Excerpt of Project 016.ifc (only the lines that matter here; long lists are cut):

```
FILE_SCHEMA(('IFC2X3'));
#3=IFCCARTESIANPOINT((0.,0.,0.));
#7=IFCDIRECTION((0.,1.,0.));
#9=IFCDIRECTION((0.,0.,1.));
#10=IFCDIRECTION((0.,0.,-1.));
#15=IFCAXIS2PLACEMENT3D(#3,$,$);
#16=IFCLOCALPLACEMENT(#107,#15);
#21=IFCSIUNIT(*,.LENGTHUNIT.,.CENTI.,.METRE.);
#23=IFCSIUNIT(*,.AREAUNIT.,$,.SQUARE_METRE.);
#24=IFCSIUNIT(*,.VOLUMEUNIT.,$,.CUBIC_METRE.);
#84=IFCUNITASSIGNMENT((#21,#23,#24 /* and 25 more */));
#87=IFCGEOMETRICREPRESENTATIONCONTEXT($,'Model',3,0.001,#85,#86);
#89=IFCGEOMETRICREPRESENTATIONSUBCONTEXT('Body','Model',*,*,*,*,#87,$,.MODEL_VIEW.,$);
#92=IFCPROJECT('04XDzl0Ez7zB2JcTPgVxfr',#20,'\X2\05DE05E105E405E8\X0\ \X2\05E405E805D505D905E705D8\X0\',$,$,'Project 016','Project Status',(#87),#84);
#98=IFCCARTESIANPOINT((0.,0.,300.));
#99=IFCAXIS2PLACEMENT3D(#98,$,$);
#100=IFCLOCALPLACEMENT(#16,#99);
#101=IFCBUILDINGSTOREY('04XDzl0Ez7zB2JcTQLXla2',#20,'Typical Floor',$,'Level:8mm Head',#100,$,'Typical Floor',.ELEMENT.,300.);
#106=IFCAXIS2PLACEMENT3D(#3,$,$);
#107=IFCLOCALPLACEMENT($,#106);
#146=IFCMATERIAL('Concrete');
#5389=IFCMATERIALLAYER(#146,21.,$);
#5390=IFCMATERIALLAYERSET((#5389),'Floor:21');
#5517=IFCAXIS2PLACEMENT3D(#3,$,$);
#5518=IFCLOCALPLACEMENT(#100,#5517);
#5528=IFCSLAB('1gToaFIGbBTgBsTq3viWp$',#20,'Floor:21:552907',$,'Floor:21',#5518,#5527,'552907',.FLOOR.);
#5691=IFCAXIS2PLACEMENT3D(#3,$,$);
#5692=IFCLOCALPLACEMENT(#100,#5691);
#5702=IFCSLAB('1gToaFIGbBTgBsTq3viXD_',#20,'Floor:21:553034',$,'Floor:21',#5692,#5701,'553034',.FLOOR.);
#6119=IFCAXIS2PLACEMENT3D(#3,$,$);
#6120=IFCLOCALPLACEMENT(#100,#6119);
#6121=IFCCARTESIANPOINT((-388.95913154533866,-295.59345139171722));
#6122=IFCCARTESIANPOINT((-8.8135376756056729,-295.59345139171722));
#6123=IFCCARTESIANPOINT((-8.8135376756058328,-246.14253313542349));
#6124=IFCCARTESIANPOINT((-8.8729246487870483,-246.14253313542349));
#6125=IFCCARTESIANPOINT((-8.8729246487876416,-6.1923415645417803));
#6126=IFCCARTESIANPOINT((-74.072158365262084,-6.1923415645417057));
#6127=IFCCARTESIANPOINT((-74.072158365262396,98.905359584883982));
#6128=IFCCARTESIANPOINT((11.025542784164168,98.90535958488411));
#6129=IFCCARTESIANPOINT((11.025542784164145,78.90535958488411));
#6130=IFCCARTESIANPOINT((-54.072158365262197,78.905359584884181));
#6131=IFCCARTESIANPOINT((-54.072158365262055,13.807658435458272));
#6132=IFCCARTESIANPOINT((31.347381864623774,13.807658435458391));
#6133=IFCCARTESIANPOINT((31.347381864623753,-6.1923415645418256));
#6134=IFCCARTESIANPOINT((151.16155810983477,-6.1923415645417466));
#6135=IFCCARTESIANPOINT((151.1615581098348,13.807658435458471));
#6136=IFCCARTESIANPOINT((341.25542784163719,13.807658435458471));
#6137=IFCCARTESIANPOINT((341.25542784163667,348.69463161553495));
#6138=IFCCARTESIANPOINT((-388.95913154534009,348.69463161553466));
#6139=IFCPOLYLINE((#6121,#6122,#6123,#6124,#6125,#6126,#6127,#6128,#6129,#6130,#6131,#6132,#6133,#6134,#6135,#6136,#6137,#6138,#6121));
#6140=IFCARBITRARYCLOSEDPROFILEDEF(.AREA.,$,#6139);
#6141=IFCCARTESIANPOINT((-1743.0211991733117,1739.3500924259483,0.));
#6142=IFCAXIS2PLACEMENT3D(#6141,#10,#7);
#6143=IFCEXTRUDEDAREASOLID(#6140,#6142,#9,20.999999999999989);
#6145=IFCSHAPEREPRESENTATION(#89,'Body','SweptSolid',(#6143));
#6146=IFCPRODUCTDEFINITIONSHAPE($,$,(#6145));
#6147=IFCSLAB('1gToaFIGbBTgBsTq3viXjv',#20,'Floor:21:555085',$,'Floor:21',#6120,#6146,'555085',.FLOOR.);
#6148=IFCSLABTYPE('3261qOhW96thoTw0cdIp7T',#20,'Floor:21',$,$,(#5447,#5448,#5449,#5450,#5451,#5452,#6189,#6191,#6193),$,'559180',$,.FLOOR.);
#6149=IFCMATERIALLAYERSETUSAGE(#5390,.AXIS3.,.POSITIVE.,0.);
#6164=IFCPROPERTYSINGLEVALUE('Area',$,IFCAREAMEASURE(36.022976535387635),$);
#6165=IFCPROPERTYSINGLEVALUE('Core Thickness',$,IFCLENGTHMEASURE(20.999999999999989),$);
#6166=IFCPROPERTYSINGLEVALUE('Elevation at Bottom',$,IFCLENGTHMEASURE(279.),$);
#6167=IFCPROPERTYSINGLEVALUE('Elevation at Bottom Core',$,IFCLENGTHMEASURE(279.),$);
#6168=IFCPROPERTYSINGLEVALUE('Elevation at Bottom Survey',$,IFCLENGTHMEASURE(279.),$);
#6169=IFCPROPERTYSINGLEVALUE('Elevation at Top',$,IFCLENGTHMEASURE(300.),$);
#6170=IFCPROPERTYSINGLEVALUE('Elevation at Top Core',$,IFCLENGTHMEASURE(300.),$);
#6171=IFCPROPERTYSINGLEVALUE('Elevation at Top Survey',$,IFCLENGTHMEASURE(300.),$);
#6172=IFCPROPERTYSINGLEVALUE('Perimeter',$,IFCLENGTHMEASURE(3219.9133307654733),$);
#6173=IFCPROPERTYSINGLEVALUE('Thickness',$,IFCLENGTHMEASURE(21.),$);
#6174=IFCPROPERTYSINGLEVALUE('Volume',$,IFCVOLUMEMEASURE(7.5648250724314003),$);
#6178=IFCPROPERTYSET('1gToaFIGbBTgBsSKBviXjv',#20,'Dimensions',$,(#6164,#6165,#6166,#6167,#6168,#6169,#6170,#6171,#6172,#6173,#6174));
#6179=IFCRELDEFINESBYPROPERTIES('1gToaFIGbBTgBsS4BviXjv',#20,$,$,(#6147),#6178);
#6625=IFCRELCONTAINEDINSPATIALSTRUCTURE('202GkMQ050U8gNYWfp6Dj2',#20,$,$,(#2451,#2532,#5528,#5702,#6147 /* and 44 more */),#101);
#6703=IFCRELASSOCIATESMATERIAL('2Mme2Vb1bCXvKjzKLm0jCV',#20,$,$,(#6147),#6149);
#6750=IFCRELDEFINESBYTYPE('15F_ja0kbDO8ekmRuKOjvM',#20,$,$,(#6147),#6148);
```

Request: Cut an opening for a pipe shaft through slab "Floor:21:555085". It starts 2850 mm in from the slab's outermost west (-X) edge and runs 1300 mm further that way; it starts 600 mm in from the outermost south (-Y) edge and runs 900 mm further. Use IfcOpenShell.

```python
import numpy as np
import ifcopenshell
import ifcopenshell.api.feature
import ifcopenshell.api.geometry
import ifcopenshell.api.pset
import ifcopenshell.api.root
import ifcopenshell.geom
import ifcopenshell.util.element
import ifcopenshell.util.placement
import ifcopenshell.util.representation
import ifcopenshell.util.shape
import ifcopenshell.util.unit

model = ifcopenshell.open("Project 016.ifc")
unit_scale = ifcopenshell.util.unit.calculate_unit_scale(model)
area_scale = ifcopenshell.util.unit.calculate_unit_scale(model, "AREAUNIT")
volume_scale = ifcopenshell.util.unit.calculate_unit_scale(model, "VOLUMEUNIT")
settings = ifcopenshell.geom.settings()


def volume(element):
    """Net volume in cubic metres, openings subtracted."""
    shape = ifcopenshell.geom.create_shape(settings, element)
    return ifcopenshell.util.shape.get_volume(shape.geometry)


slab = model.by_guid("1gToaFIGbBTgBsTq3viXjv")
before = volume(slab)

# Extent in the slab's own axes, in metres. The edges named are its -X and -Y sides.
slab_shape = ifcopenshell.geom.create_shape(settings, slab)
vertices = ifcopenshell.util.shape.get_vertices(slab_shape.geometry)
x_min, y_min, bottom = vertices.min(axis=0)
top = vertices[:, 2].max()

opening = ifcopenshell.api.root.create_entity(model, ifc_class="IfcOpeningElement", name="Pipe shaft opening")
context = ifcopenshell.util.representation.get_context(model, "Model", "Body", "MODEL_VIEW")
width, depth = 1.3, 0.9
outline = [(0.0, 0.0), (width, 0.0), (width, depth), (0.0, depth), (0.0, 0.0)]
# Overshoot both faces by 50 mm so the cut is clean.
shape = ifcopenshell.api.geometry.add_slab_representation(
    model, context=context, depth=top - bottom + 0.1, polyline=outline
)
ifcopenshell.api.geometry.assign_representation(model, product=opening, representation=shape)

matrix = ifcopenshell.util.placement.get_local_placement(slab.ObjectPlacement)
matrix[:, 3] = matrix @ np.append(np.array([x_min + 2.85, y_min + 0.6, bottom - 0.05]) / unit_scale, 1.0)
ifcopenshell.api.geometry.edit_object_placement(model, product=opening, matrix=matrix, is_si=False)
ifcopenshell.api.feature.add_feature(model, feature=opening, element=slab)

after = volume(slab)

# Update the slab's stored quantities.
pset = model.by_id(ifcopenshell.util.element.get_pset(slab, "Dimensions", should_inherit=False)["id"])
ifcopenshell.api.pset.edit_pset(model, pset=pset, properties={
    "Area": model.create_entity("IfcAreaMeasure", after / (top - bottom) / area_scale),
    "Volume": model.create_entity("IfcVolumeMeasure", after / volume_scale),
})

print(f"slab volume {before:.3f} -> {after:.3f} m3")

model.write("Project 016_edited.ifc")
```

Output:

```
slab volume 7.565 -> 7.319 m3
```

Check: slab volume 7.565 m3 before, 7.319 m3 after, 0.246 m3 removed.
